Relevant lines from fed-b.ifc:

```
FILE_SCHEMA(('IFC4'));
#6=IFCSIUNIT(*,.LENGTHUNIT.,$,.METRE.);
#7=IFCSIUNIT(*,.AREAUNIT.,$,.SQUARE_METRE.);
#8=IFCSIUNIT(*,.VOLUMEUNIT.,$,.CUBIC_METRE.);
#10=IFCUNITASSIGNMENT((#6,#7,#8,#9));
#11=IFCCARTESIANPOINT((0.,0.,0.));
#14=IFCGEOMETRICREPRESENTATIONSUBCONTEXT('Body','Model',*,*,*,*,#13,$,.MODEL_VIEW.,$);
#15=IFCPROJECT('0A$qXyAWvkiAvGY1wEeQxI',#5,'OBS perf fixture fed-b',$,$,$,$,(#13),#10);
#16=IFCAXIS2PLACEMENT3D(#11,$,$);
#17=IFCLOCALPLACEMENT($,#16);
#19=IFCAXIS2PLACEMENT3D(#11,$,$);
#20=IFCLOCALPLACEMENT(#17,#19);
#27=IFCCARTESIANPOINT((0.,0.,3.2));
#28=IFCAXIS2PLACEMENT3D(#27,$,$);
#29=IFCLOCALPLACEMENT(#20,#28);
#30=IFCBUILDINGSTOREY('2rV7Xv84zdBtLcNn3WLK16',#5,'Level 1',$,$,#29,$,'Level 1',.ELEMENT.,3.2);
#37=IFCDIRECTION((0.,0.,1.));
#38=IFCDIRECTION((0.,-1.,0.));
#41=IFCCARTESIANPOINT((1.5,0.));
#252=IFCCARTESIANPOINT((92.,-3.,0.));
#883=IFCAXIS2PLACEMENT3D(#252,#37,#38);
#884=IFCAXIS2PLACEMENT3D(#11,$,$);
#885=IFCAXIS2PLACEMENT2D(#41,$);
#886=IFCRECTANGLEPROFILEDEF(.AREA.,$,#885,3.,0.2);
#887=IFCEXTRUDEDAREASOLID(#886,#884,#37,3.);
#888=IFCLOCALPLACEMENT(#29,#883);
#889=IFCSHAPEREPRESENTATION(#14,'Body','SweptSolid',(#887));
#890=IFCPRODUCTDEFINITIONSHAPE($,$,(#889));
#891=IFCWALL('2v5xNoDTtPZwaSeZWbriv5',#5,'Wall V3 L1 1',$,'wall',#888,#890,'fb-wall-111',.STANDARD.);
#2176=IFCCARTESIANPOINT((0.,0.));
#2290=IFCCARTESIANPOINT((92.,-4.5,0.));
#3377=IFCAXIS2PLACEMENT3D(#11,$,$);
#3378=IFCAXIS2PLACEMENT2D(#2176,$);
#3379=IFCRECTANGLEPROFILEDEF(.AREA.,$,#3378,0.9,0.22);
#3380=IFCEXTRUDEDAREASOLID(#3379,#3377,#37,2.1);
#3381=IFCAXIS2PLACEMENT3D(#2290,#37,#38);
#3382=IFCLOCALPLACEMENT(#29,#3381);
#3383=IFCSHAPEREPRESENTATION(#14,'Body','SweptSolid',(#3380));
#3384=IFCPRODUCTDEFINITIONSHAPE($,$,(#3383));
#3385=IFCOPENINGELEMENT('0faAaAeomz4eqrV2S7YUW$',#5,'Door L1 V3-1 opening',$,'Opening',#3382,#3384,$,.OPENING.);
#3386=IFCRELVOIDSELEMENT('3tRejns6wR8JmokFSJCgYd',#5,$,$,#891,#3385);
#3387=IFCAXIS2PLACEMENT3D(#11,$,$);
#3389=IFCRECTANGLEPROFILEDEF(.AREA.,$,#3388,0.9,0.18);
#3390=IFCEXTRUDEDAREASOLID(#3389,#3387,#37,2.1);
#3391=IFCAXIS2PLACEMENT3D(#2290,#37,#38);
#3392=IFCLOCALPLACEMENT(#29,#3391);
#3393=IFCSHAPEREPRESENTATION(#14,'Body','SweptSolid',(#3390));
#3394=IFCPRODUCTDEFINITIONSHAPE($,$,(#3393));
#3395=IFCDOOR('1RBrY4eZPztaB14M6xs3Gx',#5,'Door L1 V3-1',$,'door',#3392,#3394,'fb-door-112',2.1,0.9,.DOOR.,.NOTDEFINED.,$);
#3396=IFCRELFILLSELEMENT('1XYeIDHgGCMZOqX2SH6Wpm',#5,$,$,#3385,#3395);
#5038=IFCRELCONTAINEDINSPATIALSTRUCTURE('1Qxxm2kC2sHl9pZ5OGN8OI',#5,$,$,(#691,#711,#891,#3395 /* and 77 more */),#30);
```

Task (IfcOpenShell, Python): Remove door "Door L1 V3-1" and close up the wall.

```python
import ifcopenshell
import ifcopenshell.api.feature
import ifcopenshell.api.root
import ifcopenshell.geom
import ifcopenshell.util.shape

model = ifcopenshell.open("fed-b.ifc")
settings = ifcopenshell.geom.settings()


def volume(element):
    """Net volume in cubic metres, openings subtracted."""
    shape = ifcopenshell.geom.create_shape(settings, element)
    return ifcopenshell.util.shape.get_volume(shape.geometry)


door = model.by_id(3395)
opening = door.FillsVoids[0].RelatingOpeningElement
wall = opening.VoidsElements[0].RelatingBuildingElement
before = volume(wall)

ifcopenshell.api.root.remove_product(model, product=door)
ifcopenshell.api.feature.remove_feature(model, feature=opening)

after = volume(wall)

print(f"wall volume {before:.3f} -> {after:.3f} m3")

model.write("fed-b-out.ifc")
```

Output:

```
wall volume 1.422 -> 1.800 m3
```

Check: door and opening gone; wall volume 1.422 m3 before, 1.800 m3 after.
